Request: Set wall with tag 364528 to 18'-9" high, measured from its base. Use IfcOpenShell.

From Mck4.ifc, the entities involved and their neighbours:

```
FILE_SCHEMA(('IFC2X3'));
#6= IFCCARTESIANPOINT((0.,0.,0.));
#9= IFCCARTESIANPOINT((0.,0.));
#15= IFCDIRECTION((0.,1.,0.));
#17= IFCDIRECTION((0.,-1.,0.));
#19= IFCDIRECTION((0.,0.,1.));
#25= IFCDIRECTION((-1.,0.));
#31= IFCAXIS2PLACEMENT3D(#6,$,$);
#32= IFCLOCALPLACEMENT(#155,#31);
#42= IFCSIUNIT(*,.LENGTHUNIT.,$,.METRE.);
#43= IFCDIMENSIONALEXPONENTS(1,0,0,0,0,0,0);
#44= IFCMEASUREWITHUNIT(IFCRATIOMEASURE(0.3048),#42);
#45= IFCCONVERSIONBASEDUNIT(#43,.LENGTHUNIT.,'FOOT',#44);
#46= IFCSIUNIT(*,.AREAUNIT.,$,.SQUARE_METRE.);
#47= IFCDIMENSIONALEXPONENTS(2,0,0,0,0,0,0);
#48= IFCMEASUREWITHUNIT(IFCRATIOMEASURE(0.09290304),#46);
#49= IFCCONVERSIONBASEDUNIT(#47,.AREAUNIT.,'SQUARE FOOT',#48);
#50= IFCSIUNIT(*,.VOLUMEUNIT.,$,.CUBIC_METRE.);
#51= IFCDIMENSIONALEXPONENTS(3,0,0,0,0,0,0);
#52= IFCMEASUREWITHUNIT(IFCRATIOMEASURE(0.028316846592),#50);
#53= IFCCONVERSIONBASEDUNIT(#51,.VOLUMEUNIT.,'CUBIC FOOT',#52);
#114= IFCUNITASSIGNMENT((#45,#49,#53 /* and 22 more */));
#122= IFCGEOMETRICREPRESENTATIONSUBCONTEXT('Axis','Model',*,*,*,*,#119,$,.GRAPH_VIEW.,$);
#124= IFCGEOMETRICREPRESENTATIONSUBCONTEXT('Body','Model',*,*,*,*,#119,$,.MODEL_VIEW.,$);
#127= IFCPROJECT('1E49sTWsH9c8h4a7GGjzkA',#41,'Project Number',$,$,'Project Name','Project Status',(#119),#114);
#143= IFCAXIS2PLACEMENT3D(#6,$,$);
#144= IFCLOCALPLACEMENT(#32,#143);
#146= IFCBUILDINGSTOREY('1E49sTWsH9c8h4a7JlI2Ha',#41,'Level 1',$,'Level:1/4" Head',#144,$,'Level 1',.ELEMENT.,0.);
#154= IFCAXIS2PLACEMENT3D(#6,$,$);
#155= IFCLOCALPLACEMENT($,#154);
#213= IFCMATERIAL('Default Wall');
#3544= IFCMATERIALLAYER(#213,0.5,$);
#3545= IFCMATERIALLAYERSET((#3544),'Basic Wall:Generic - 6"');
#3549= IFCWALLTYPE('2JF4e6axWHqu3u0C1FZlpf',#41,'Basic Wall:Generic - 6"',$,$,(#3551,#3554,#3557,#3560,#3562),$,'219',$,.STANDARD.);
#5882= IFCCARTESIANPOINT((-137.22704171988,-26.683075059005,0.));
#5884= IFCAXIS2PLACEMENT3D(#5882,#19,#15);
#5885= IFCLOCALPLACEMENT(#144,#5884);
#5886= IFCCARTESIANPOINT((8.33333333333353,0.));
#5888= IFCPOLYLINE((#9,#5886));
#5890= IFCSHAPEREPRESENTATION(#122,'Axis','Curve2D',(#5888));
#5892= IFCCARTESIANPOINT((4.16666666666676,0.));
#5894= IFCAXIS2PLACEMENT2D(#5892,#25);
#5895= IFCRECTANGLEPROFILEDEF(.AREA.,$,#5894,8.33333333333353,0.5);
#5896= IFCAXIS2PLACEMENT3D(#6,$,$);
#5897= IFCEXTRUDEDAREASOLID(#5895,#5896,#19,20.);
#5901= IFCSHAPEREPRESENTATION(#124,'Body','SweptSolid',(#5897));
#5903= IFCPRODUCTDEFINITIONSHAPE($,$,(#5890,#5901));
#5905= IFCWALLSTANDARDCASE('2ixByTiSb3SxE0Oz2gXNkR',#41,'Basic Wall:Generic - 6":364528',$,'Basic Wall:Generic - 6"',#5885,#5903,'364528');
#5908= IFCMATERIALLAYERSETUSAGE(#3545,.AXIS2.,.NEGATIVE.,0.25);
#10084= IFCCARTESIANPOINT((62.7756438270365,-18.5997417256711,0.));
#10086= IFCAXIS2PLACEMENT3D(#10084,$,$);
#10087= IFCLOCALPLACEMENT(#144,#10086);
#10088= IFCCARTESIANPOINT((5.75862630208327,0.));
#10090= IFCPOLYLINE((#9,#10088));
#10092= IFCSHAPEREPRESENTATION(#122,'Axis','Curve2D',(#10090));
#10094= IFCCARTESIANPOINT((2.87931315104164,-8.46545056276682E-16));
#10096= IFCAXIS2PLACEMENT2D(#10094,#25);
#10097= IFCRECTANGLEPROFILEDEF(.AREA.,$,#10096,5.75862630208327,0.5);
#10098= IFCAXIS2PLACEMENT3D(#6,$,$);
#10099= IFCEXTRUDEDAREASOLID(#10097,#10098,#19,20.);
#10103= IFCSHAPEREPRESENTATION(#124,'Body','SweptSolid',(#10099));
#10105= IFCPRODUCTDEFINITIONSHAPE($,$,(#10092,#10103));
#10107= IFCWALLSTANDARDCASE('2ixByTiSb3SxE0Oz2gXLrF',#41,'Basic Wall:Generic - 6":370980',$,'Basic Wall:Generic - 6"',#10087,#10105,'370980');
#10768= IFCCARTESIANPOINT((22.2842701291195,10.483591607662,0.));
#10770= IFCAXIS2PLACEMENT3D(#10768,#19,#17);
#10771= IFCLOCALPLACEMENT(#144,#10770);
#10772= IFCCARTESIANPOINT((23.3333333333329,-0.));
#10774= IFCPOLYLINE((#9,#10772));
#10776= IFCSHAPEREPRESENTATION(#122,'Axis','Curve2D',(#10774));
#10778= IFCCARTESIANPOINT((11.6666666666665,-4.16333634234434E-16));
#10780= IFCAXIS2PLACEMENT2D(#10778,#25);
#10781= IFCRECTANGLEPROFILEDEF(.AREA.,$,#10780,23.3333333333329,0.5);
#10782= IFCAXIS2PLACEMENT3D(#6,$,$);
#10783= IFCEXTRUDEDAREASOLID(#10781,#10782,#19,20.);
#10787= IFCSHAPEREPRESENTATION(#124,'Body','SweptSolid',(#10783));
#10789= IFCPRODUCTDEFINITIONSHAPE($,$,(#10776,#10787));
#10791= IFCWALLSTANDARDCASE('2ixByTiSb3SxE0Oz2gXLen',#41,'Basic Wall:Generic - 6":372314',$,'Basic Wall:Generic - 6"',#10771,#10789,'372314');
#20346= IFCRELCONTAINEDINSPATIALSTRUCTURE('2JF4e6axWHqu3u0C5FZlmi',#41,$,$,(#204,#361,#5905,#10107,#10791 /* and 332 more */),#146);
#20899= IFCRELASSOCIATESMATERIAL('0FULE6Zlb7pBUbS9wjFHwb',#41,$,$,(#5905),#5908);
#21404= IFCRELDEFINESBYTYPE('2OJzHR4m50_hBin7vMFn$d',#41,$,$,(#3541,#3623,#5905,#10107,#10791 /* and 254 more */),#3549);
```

```python
import ifcopenshell
import ifcopenshell.geom
import ifcopenshell.util.representation
import ifcopenshell.util.shape
import ifcopenshell.util.unit

model = ifcopenshell.open("Mck4.ifc")
unit_scale = ifcopenshell.util.unit.calculate_unit_scale(model)
settings = ifcopenshell.geom.settings()


def volume(element):
    """Net volume in cubic metres, openings subtracted."""
    shape = ifcopenshell.geom.create_shape(settings, element)
    return ifcopenshell.util.shape.get_volume(shape.geometry)


wall = model.by_id(5905)
before = volume(wall)

body = ifcopenshell.util.representation.get_representation(wall, "Model", "Body")
solid = body.Items[0]
old_height = solid.Depth
solid.Depth = 225 * 0.0254 / unit_scale
after = volume(wall)

print(f"height {old_height:g} -> {solid.Depth:g}, volume {before:.3f} -> {after:.3f} m3")

model.write("Mck4_rev.ifc")
```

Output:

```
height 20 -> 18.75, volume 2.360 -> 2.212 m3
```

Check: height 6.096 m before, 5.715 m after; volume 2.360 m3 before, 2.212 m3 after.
